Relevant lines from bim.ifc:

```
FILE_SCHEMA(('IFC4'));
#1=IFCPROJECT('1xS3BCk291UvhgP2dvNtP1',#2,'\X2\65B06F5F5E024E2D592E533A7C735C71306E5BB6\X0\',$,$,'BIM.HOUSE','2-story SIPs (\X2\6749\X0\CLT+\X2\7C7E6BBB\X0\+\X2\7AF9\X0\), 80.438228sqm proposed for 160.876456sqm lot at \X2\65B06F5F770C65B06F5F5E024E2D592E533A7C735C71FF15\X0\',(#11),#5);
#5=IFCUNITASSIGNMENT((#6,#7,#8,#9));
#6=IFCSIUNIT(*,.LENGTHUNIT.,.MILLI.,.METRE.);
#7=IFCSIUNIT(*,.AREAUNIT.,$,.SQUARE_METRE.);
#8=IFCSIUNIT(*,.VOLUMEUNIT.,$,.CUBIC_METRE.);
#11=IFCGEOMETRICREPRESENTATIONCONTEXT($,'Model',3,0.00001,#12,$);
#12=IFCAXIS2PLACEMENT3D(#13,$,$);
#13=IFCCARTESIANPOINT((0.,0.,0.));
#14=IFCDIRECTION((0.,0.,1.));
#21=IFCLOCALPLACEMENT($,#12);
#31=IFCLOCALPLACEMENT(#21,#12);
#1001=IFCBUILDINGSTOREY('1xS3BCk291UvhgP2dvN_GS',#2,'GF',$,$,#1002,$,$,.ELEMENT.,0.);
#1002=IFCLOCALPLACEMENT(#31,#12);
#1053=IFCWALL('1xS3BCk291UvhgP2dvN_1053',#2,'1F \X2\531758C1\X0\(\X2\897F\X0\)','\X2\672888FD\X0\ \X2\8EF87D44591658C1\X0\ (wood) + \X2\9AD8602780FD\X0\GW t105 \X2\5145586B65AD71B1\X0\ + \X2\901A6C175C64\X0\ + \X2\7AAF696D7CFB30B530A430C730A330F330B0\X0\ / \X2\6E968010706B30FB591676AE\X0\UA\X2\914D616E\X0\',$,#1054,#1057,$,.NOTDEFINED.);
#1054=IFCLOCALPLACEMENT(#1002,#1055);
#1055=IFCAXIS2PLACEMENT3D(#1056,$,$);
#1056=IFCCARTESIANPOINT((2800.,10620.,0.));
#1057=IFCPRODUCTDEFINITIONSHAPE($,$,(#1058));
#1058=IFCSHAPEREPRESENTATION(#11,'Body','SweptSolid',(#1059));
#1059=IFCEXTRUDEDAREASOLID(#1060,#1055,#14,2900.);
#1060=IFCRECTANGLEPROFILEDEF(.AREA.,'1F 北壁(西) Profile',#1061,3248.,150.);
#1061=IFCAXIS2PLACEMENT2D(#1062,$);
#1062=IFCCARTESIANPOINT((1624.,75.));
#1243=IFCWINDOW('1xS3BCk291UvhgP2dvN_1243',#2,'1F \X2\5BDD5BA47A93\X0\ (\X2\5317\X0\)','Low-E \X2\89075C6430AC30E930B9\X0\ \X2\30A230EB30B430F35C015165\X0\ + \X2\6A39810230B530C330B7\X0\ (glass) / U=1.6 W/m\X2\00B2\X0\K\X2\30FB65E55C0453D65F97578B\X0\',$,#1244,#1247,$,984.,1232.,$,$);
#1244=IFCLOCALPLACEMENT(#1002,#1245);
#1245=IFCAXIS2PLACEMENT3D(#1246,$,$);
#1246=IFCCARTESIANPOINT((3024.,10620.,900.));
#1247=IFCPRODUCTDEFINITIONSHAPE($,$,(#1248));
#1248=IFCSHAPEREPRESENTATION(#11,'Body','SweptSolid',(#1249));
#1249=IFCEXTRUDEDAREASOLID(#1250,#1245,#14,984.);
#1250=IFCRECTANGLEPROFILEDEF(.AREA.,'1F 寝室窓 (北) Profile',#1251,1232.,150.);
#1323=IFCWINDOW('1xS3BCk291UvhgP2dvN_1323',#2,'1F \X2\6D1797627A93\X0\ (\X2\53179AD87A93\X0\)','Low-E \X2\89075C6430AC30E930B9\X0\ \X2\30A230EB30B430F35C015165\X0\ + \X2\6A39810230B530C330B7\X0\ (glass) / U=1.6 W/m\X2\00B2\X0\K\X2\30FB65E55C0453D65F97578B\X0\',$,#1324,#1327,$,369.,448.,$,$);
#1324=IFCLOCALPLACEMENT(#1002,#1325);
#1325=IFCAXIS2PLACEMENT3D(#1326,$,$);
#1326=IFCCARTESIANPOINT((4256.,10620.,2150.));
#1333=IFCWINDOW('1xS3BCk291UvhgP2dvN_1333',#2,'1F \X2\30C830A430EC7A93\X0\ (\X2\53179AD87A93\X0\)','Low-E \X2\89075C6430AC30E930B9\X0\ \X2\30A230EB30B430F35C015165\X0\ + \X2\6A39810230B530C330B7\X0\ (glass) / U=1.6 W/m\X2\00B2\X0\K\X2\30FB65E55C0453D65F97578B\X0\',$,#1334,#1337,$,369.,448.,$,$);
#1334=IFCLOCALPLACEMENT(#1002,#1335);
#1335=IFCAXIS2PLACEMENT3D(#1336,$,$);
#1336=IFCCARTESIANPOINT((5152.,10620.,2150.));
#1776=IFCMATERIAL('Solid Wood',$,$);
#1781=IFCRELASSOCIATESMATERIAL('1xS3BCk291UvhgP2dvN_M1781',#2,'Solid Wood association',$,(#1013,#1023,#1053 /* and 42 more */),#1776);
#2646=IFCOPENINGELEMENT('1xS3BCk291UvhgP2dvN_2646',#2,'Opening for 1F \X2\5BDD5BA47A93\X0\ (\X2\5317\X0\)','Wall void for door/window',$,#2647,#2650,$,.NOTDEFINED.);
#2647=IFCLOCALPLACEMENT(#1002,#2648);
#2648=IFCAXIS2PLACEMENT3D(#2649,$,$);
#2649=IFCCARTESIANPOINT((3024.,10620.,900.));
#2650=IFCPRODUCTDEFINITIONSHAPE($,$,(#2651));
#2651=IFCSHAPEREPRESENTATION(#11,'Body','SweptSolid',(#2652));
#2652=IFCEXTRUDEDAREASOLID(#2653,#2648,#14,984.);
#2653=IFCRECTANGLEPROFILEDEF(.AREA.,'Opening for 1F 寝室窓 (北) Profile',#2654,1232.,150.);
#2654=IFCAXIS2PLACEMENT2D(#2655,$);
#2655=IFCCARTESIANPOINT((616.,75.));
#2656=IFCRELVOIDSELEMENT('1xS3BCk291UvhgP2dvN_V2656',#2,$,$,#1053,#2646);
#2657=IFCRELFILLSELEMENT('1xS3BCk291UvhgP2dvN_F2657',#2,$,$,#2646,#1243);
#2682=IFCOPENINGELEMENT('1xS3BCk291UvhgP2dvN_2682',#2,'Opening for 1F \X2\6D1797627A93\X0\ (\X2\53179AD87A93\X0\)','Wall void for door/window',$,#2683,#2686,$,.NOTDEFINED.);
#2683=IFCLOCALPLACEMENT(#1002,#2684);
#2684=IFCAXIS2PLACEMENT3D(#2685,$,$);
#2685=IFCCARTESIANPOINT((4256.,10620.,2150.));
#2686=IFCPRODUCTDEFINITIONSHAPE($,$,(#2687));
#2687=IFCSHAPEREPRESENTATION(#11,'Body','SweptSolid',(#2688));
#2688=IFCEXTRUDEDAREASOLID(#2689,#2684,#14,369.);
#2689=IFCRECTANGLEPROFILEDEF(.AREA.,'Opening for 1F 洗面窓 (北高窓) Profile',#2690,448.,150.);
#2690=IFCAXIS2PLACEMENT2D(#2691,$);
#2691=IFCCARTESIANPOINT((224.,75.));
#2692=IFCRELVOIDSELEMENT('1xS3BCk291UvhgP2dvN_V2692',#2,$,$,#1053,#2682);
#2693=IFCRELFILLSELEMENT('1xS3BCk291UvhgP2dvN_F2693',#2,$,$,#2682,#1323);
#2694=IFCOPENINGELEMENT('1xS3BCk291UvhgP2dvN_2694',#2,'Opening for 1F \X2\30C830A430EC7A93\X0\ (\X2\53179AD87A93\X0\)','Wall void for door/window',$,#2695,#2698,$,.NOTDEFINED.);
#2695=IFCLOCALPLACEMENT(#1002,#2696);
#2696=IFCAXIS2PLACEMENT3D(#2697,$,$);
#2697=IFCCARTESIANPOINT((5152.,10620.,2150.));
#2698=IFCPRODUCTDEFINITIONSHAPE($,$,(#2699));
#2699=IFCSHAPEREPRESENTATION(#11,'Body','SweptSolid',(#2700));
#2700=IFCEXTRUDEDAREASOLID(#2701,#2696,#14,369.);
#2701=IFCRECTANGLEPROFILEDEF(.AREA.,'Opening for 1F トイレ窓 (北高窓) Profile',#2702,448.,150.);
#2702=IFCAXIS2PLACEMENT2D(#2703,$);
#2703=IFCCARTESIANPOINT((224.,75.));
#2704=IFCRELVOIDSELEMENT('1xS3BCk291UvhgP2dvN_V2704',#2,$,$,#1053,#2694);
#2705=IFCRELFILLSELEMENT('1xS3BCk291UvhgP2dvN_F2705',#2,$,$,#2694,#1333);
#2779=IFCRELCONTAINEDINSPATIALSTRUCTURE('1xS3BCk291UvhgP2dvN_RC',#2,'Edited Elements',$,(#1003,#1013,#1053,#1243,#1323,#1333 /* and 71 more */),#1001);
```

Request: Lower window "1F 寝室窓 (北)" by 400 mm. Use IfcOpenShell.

```python
import numpy as np
import ifcopenshell
import ifcopenshell.api.geometry
import ifcopenshell.util.placement
import ifcopenshell.util.unit

model = ifcopenshell.open("bim.ifc")
unit_scale = ifcopenshell.util.unit.calculate_unit_scale(model)

window = model.by_id(1243)
opening = window.FillsVoids[0].RelatingOpeningElement
dz = -400.0

shift = np.array([0.0, 0.0, dz])
# The window is not placed relative to its opening, so move both.
for product in (opening, window):
    matrix = ifcopenshell.util.placement.get_local_placement(product.ObjectPlacement)
    matrix[:3, 3] += shift
    ifcopenshell.api.geometry.edit_object_placement(model, product=product, matrix=matrix, is_si=False)

print(f"moved by {dz * unit_scale:+.3f} m")

model.write("bim_v2.ifc")
```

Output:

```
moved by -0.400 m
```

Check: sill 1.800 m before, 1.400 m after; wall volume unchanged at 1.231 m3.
